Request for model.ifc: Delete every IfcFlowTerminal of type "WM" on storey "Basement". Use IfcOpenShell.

First a look at what the model holds.

```python
import ifcopenshell
import ifcopenshell.util.element

model = ifcopenshell.open("model.ifc")
print(model.schema)
storey = next(s for s in model.by_type("IfcBuildingStorey") if s.Name == "Basement")
terminals = [e for e in ifcopenshell.util.element.get_decomposition(storey) if e.is_a("IfcFlowTerminal")]
seen = {}
for e in terminals:
    element_type = ifcopenshell.util.element.get_type(e)
    name = element_type.Name if element_type not in (None, e) else None
    seen[name] = seen.get(name, 0) + 1
for name, count in sorted(seen.items(), key=str):
    print(count, "x", name)
```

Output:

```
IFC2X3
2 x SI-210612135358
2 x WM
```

```python
import ifcopenshell
import ifcopenshell.api.root
import ifcopenshell.util.element

model = ifcopenshell.open("model.ifc")

storey = next(s for s in model.by_type("IfcBuildingStorey") if s.Name == "Basement")
terminals = [e for e in ifcopenshell.util.element.get_decomposition(storey) if e.is_a("IfcFlowTerminal")]
targets = [e for e in terminals if (t := ifcopenshell.util.element.get_type(e)) not in (None, e) and t.Name == "WM"]

for e in targets:
    ifcopenshell.api.root.remove_product(model, product=e)
print(len(targets), "removed")

model.write("model_v2.ifc")
```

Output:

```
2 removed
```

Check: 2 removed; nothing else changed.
